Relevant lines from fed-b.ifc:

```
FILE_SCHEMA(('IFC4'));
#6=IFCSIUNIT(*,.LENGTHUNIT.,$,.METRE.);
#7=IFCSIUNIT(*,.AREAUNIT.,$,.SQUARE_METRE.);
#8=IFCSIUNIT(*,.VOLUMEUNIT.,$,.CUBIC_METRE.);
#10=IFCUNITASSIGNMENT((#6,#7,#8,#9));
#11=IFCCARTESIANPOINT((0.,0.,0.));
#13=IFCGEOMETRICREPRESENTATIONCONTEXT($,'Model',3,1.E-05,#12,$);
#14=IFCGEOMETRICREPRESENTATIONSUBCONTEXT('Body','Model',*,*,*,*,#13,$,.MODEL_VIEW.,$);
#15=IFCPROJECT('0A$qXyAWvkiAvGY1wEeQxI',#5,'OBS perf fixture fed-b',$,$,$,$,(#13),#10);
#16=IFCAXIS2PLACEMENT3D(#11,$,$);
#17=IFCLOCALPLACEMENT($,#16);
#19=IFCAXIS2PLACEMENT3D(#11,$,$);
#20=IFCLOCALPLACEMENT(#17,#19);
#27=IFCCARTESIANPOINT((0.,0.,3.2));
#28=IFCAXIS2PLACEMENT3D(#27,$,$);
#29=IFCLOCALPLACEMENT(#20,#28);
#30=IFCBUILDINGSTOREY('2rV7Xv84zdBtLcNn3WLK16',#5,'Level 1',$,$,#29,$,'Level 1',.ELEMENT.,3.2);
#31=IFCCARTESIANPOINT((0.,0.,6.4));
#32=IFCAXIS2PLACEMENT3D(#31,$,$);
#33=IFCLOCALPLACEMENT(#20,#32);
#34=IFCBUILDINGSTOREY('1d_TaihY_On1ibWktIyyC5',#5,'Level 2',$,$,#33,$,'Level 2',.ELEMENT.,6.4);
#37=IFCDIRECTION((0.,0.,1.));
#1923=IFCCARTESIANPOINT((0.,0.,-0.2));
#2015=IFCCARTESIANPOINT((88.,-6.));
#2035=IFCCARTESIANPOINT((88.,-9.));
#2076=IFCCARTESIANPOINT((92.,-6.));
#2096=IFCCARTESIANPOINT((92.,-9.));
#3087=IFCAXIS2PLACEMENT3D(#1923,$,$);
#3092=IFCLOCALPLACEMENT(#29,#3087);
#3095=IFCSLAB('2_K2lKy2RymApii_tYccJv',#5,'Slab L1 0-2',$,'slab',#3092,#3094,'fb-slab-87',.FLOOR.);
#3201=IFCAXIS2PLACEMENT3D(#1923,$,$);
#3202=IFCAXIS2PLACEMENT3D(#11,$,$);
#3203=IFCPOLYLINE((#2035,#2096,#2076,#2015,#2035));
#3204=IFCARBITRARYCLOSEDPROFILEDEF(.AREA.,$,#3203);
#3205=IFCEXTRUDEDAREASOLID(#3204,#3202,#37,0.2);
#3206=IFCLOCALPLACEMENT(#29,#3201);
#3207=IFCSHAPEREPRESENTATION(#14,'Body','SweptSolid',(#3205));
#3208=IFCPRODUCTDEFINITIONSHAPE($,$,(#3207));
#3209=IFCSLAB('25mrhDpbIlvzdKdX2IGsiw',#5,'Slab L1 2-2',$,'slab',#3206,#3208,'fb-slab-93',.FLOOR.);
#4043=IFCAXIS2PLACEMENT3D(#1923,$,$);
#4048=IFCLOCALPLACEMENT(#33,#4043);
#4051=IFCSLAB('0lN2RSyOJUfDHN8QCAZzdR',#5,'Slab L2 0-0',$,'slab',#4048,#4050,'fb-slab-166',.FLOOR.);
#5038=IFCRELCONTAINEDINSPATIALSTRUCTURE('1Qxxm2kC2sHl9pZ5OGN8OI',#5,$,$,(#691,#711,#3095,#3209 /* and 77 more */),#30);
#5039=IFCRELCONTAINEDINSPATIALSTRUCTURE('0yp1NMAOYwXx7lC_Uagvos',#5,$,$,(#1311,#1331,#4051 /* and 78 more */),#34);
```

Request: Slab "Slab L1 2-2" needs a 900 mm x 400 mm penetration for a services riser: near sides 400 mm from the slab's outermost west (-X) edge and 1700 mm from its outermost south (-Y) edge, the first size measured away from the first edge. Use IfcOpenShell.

```python
import numpy as np
import ifcopenshell
import ifcopenshell.api.feature
import ifcopenshell.api.geometry
import ifcopenshell.api.root
import ifcopenshell.geom
import ifcopenshell.util.placement
import ifcopenshell.util.representation
import ifcopenshell.util.shape
import ifcopenshell.util.unit

model = ifcopenshell.open("fed-b.ifc")
unit_scale = ifcopenshell.util.unit.calculate_unit_scale(model)
settings = ifcopenshell.geom.settings()


def volume(element):
    """Net volume in cubic metres, openings subtracted."""
    shape = ifcopenshell.geom.create_shape(settings, element)
    return ifcopenshell.util.shape.get_volume(shape.geometry)


slab = model.by_guid("25mrhDpbIlvzdKdX2IGsiw")
before = volume(slab)

# Extent in the slab's own axes, in metres. The edges named are its -X and -Y sides.
slab_shape = ifcopenshell.geom.create_shape(settings, slab)
vertices = ifcopenshell.util.shape.get_vertices(slab_shape.geometry)
x_min, y_min, bottom = vertices.min(axis=0)
top = vertices[:, 2].max()

opening = ifcopenshell.api.root.create_entity(model, ifc_class="IfcOpeningElement", name="Services riser opening", predefined_type="OPENING")
context = ifcopenshell.util.representation.get_context(model, "Model", "Body", "MODEL_VIEW")
width, depth = 0.9, 0.4
outline = [(0.0, 0.0), (width, 0.0), (width, depth), (0.0, depth), (0.0, 0.0)]
# Overshoot both faces by 50 mm so the cut is clean.
shape = ifcopenshell.api.geometry.add_slab_representation(
    model, context=context, depth=top - bottom + 0.1, polyline=outline
)
ifcopenshell.api.geometry.assign_representation(model, product=opening, representation=shape)

matrix = ifcopenshell.util.placement.get_local_placement(slab.ObjectPlacement)
matrix[:, 3] = matrix @ np.append(np.array([x_min + 0.4, y_min + 1.7, bottom - 0.05]) / unit_scale, 1.0)
ifcopenshell.api.geometry.edit_object_placement(model, product=opening, matrix=matrix, is_si=False)
ifcopenshell.api.feature.add_feature(model, feature=opening, element=slab)

after = volume(slab)

print(f"slab volume {before:.3f} -> {after:.3f} m3")

model.write("fed-b-out.ifc")
```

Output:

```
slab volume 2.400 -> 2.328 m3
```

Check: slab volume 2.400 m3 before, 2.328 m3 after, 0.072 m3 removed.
